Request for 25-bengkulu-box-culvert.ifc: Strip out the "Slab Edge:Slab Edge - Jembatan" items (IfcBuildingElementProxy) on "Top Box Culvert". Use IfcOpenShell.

First a look at what the model holds.

```python
import ifcopenshell
import ifcopenshell.util.element

model = ifcopenshell.open("25-bengkulu-box-culvert.ifc")
print(model.schema)
storey = next(s for s in model.by_type("IfcBuildingStorey") if s.Name == "Top Box Culvert")
proxies = [e for e in ifcopenshell.util.element.get_decomposition(storey) if e.is_a("IfcBuildingElementProxy")]
seen = {}
for e in proxies:
    element_type = ifcopenshell.util.element.get_type(e)
    name = element_type.Name if element_type not in (None, e) else None
    seen[name] = seen.get(name, 0) + 1
for name, count in sorted(seen.items(), key=str):
    print(count, "x", name)
```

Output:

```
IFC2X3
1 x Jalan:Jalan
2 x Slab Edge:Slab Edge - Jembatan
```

```python
import ifcopenshell
import ifcopenshell.api.root
import ifcopenshell.util.element

model = ifcopenshell.open("25-bengkulu-box-culvert.ifc")

storey = next(s for s in model.by_type("IfcBuildingStorey") if s.Name == "Top Box Culvert")
proxies = [e for e in ifcopenshell.util.element.get_decomposition(storey) if e.is_a("IfcBuildingElementProxy")]
targets = [e for e in proxies if (t := ifcopenshell.util.element.get_type(e)) not in (None, e) and t.Name == "Slab Edge:Slab Edge - Jembatan"]

for e in targets:
    ifcopenshell.api.root.remove_product(model, product=e)
print(len(targets), "removed")

model.write("25-bengkulu-box-culvert_edited.ifc")
```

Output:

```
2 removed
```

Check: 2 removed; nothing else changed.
